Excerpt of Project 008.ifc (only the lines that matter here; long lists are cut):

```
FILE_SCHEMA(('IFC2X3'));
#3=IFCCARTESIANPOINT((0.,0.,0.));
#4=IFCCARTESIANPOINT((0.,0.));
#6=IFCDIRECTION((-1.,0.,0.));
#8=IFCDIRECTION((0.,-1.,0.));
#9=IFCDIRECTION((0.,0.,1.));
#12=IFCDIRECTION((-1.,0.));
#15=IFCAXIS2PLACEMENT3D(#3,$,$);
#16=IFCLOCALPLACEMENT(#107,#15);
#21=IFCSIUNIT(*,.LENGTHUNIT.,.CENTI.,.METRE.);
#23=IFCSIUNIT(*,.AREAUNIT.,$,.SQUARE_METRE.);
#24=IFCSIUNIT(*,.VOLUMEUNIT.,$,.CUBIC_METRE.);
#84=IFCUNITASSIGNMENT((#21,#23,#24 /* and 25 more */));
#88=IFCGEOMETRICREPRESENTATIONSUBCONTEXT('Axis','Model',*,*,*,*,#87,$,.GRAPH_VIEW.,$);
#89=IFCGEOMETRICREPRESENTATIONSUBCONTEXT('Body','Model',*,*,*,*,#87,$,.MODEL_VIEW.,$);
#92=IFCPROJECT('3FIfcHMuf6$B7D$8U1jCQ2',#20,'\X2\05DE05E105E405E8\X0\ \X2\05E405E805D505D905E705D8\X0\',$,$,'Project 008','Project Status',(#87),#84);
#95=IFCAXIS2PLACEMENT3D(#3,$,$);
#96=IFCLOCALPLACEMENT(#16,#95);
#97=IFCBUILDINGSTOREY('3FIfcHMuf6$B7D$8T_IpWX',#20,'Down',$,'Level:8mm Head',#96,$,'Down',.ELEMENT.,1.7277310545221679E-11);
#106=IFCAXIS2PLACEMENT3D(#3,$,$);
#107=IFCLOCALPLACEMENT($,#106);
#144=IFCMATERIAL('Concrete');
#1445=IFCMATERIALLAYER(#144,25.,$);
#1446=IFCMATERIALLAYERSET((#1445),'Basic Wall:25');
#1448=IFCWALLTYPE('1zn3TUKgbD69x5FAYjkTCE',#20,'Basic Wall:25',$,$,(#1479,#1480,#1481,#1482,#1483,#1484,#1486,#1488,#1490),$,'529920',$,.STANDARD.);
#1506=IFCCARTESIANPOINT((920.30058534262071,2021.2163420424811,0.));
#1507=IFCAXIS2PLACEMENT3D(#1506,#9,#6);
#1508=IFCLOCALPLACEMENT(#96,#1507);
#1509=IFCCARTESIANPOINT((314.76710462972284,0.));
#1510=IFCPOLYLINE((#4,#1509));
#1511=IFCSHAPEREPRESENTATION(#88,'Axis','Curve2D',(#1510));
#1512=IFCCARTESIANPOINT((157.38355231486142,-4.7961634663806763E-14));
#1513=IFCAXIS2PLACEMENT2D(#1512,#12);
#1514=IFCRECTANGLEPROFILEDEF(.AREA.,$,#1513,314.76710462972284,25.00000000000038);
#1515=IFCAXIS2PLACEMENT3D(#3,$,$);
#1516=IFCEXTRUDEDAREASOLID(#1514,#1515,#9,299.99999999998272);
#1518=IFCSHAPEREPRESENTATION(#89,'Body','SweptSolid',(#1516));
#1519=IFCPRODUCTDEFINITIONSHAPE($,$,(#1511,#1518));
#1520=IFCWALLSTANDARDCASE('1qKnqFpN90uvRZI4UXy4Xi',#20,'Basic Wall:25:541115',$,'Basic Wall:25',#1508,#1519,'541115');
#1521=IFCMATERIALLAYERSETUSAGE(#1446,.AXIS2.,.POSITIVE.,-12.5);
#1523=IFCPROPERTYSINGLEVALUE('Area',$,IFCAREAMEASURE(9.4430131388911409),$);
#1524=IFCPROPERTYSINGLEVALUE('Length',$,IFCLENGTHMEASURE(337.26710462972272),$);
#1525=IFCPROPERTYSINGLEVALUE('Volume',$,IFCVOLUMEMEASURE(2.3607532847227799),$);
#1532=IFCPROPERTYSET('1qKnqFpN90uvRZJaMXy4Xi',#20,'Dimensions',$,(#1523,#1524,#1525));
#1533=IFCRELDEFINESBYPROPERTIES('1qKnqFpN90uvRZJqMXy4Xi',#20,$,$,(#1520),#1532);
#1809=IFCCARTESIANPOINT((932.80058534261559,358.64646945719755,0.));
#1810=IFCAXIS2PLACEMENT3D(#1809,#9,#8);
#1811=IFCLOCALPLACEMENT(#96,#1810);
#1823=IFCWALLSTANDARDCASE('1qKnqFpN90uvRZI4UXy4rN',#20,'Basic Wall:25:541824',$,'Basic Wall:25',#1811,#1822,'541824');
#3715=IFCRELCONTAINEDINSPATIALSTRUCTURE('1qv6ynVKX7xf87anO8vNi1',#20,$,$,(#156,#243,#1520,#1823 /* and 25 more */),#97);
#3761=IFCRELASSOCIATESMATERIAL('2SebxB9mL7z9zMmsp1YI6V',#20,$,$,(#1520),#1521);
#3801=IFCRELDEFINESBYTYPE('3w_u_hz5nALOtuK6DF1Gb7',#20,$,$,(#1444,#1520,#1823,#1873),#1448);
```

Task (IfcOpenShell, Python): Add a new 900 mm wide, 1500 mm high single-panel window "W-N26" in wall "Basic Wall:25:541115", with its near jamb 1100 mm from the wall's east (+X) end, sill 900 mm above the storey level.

```python
import numpy as np
import ifcopenshell
import ifcopenshell.api.feature
import ifcopenshell.api.geometry
import ifcopenshell.api.pset
import ifcopenshell.api.root
import ifcopenshell.api.spatial
import ifcopenshell.api.type
import ifcopenshell.geom
import ifcopenshell.util.element
import ifcopenshell.util.placement
import ifcopenshell.util.representation
import ifcopenshell.util.shape
import ifcopenshell.util.unit

model = ifcopenshell.open("Project 008.ifc")
unit_scale = ifcopenshell.util.unit.calculate_unit_scale(model)
area_scale = ifcopenshell.util.unit.calculate_unit_scale(model, "AREAUNIT")
volume_scale = ifcopenshell.util.unit.calculate_unit_scale(model, "VOLUMEUNIT")
settings = ifcopenshell.geom.settings()


def volume(element):
    """Net volume in cubic metres, openings subtracted."""
    shape = ifcopenshell.geom.create_shape(settings, element)
    return ifcopenshell.util.shape.get_volume(shape.geometry)


wall = model.by_guid("1qKnqFpN90uvRZI4UXy4Xi")
storey = ifcopenshell.util.element.get_container(wall, ifc_class="IfcBuildingStorey")
context = ifcopenshell.util.representation.get_context(model, "Model", "Body", "MODEL_VIEW")
before = volume(wall)

width, height, from_end, sill = 0.9, 1.5, 1.1, 0.9  # metres

# The wall runs along its own X axis, and the end named is its -X end.
wall_shape = ifcopenshell.geom.create_shape(settings, wall)
x, y, z = ifcopenshell.util.shape.get_vertices(wall_shape.geometry).T
start = x.min() + from_end
face, thickness = float(y.min()), float(y.max() - y.min())
wall_matrix = ifcopenshell.util.placement.get_local_placement(wall.ObjectPlacement)
level = ifcopenshell.util.placement.get_local_placement(storey.ObjectPlacement)[2, 3]


def in_wall(x, y):
    """Placement at x, y metres in the wall's axes, at sill height."""
    matrix = wall_matrix.copy()
    matrix[:, 3] = wall_matrix @ np.array([x / unit_scale, y / unit_scale, 0.0, 1.0])
    matrix[2, 3] = level + sill / unit_scale
    return matrix


# Opening: a box that overshoots both wall faces by 50 mm.
opening = ifcopenshell.api.root.create_entity(model, ifc_class="IfcOpeningElement")
box = ifcopenshell.api.geometry.add_wall_representation(
    model, context=context, length=width, height=height, thickness=thickness + 0.1
)
ifcopenshell.api.geometry.assign_representation(model, product=opening, representation=box)
ifcopenshell.api.geometry.edit_object_placement(model, product=opening, matrix=in_wall(start, face - 0.05), is_si=False)
ifcopenshell.api.feature.add_feature(model, feature=opening, element=wall)

window = ifcopenshell.api.root.create_entity(model, ifc_class="IfcWindow", name="W-N26")
window.OverallWidth, window.OverallHeight = width / unit_scale, height / unit_scale
body = ifcopenshell.api.geometry.add_window_representation(
    model,
    context=context,
    overall_width=window.OverallWidth,
    overall_height=window.OverallHeight,
    partition_type="SINGLE_PANEL",
)
ifcopenshell.api.geometry.assign_representation(model, product=window, representation=body)
ifcopenshell.api.spatial.assign_container(model, products=[window], relating_structure=storey)
fills = ifcopenshell.api.feature.add_filling(model, opening=opening, element=window)
fills.OwnerHistory = window.OwnerHistory  # required in IFC2X3

# IFC2X3 keeps the operation on the window style.
style = ifcopenshell.api.root.create_entity(model, ifc_class="IfcWindowStyle", name="W-N26")
style.OperationType, style.ConstructionType = "SINGLE_PANEL", "NOTDEFINED"
style.ParameterTakesPrecedence = style.Sizeable = False
ifcopenshell.api.type.assign_type(model, related_objects=[window], relating_type=style)

# Centre the window in the wall's thickness.
ifcopenshell.api.geometry.edit_object_placement(model, product=window, matrix=in_wall(start, face), is_si=False)
window_shape = ifcopenshell.geom.create_shape(settings, window)
depth = ifcopenshell.util.shape.get_vertices(window_shape.geometry)[:, 1]
offset = face + thickness / 2 - (depth.min() + depth.max()) / 2
ifcopenshell.api.geometry.edit_object_placement(model, product=window, matrix=in_wall(start, offset), is_si=False)

after = volume(wall)

# Update the wall's stored quantities.
pset = model.by_id(ifcopenshell.util.element.get_pset(wall, "Dimensions", should_inherit=False)["id"])
ifcopenshell.api.pset.edit_pset(model, pset=pset, properties={
    "Area": model.create_entity("IfcAreaMeasure", after / thickness / area_scale),
    "Volume": model.create_entity("IfcVolumeMeasure", after / volume_scale),
})

print(f"wall volume {before:.3f} -> {after:.3f} m3")

model.write("Project 008-out.ifc")
```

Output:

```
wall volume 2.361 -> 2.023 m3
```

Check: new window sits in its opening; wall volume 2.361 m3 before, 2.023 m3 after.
